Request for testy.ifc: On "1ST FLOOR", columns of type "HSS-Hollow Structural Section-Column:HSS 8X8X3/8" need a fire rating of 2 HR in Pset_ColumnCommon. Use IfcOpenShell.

First a look at what the model holds.

```python
import ifcopenshell
import ifcopenshell.util.element

model = ifcopenshell.open("testy.ifc")
print(model.schema)
storey = next(s for s in model.by_type("IfcBuildingStorey") if s.Name == "1ST FLOOR")
columns = [e for e in ifcopenshell.util.element.get_decomposition(storey) if e.is_a("IfcColumn")]
seen = {}
for e in columns:
    element_type = ifcopenshell.util.element.get_type(e)
    key = (element_type.Name if element_type != e and element_type else None, ifcopenshell.util.element.get_pset(e, "Pset_ColumnCommon", "FireRating"))
    seen[key] = seen.get(key, 0) + 1
for (name, value), count in sorted(seen.items(), key=str):
    print(count, "x", name, "|", value)
```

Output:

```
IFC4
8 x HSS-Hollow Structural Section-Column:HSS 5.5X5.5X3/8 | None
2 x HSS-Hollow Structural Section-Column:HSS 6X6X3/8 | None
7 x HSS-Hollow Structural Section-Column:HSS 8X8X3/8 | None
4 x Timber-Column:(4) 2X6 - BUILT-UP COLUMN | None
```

```python
import ifcopenshell
import ifcopenshell.api.pset
import ifcopenshell.util.element

model = ifcopenshell.open("testy.ifc")

storey = next(s for s in model.by_type("IfcBuildingStorey") if s.Name == "1ST FLOOR")
columns = [e for e in ifcopenshell.util.element.get_decomposition(storey) if e.is_a("IfcColumn")]

count = 0
for e in columns:
    element_type = ifcopenshell.util.element.get_type(e)
    if element_type in (None, e) or element_type.Name != "HSS-Hollow Structural Section-Column:HSS 8X8X3/8":
        continue
    # add_pset returns the element's existing set when there is one.
    pset = ifcopenshell.api.pset.add_pset(model, product=e, name="Pset_ColumnCommon")
    ifcopenshell.api.pset.edit_pset(model, pset=pset, properties={"FireRating": "2 HR"})
    count += 1

print(count, "columns updated")

model.write("testy_rev.ifc")
```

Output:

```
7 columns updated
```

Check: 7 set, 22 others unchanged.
